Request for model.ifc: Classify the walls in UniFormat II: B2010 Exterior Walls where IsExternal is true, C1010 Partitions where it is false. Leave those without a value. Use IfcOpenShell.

First a look at what the model holds.

```python
import ifcopenshell
import ifcopenshell.util.element

model = ifcopenshell.open("model.ifc")
print(model.schema)
print("classifications:", [c.Name for c in model.by_type("IfcClassification")])
values = [ifcopenshell.util.element.get_pset(e, "Pset_WallCommon", "IsExternal") for e in model.by_type("IfcWall")]
for value in (True, False, None):
    print("IsExternal", value, values.count(value))
```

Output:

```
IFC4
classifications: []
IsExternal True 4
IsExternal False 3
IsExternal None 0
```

```python
import ifcopenshell
import ifcopenshell.api.classification
import ifcopenshell.util.element

model = ifcopenshell.open("model.ifc")

system = ifcopenshell.api.classification.add_classification(model, classification="UniFormat II")

walls = model.by_type("IfcWall")
external = {e: ifcopenshell.util.element.get_pset(e, "Pset_WallCommon", "IsExternal") for e in walls}
for flag, code, name in ((True, "B2010", "Exterior Walls"), (False, "C1010", "Partitions")):
    products = [e for e in walls if external[e] is flag]
    ifcopenshell.api.classification.add_reference(
        model, products=products, classification=system, identification=code, name=name
    )
    print(code, len(products))

model.write("model_rev.ifc")
```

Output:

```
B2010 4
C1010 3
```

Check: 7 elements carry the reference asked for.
